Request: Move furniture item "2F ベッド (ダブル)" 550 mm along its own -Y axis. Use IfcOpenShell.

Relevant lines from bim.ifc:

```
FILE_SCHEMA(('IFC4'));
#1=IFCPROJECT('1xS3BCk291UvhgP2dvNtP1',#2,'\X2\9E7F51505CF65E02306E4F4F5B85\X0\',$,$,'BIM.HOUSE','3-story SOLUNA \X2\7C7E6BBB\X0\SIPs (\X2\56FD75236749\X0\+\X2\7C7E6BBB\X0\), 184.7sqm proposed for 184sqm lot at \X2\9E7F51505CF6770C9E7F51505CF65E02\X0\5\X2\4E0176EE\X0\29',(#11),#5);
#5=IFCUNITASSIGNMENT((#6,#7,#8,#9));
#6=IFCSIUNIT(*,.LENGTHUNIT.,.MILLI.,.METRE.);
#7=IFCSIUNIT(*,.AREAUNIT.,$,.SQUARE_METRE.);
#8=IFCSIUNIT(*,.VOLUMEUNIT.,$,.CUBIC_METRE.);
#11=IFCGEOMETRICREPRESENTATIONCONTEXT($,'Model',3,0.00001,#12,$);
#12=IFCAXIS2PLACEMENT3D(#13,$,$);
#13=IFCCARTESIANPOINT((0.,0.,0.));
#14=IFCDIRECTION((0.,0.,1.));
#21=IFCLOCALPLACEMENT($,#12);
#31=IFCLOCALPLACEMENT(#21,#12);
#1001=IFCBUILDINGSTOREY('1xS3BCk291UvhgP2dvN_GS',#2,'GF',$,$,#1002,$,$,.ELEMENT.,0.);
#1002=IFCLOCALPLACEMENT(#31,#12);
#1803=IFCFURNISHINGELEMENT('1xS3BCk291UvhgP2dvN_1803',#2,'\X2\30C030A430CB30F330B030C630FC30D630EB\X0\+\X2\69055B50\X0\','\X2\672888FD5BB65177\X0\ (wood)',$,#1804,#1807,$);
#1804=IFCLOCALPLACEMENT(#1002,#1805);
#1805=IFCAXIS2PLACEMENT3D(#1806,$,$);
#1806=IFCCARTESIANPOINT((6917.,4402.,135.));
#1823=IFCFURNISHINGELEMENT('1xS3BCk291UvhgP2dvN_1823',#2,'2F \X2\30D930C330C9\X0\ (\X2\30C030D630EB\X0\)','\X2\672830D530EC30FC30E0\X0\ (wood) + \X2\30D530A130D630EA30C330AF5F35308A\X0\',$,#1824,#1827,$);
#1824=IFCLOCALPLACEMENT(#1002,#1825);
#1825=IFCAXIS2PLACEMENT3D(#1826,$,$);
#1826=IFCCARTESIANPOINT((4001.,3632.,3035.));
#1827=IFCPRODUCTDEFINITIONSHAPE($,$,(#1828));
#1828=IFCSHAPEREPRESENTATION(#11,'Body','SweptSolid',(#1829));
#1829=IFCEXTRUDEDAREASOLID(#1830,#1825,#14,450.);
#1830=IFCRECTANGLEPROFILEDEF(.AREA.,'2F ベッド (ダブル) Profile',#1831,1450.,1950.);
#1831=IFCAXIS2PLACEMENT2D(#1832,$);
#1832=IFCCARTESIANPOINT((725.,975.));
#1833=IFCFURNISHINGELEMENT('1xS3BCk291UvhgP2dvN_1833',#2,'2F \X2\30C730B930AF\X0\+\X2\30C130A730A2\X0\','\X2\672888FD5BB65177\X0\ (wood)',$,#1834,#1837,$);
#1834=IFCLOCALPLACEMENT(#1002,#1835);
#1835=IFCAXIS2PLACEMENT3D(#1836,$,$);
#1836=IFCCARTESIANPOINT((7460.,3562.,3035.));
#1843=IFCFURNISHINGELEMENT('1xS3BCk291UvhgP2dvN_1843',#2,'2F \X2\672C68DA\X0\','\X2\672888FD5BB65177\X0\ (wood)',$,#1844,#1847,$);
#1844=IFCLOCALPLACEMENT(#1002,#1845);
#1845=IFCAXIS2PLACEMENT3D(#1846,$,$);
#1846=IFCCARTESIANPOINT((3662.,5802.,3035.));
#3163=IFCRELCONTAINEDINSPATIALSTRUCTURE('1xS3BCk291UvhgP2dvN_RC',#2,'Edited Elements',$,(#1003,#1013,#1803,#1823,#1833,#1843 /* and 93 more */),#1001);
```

```python
import ifcopenshell
import ifcopenshell.api.geometry
import ifcopenshell.util.placement
import ifcopenshell.util.unit

model = ifcopenshell.open("bim.ifc")
unit_scale = ifcopenshell.util.unit.calculate_unit_scale(model)

item = model.by_guid("1xS3BCk291UvhgP2dvN_1823")
matrix = ifcopenshell.util.placement.get_local_placement(item.ObjectPlacement)
matrix[:3, 3] -= matrix[:3, 1] * 0.55 / unit_scale
ifcopenshell.api.geometry.edit_object_placement(model, product=item, matrix=matrix, is_si=False)

print(ifcopenshell.util.placement.get_local_placement(item.ObjectPlacement).round(3) + 0.0)

model.write("bim_v2.ifc")
```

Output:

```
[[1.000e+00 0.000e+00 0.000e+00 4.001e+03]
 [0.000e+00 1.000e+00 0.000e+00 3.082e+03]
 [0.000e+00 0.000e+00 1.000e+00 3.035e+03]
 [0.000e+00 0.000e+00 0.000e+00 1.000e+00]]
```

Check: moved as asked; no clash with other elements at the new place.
